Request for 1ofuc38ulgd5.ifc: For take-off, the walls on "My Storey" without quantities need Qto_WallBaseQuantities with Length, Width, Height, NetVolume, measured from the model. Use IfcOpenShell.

First a look at what the model holds.

```python
import ifcopenshell
import ifcopenshell.util.element
import ifcopenshell.util.unit

model = ifcopenshell.open("1ofuc38ulgd5.ifc")
print(model.schema)
for unit_type in ("LENGTHUNIT", "AREAUNIT", "VOLUMEUNIT"):
    print(unit_type, ifcopenshell.util.unit.calculate_unit_scale(model, unit_type))
storey = next(s for s in model.by_type("IfcBuildingStorey") if s.Name == "My Storey")
walls = [e for e in ifcopenshell.util.element.get_decomposition(storey) if e.is_a("IfcWall")]
for e in sorted(walls, key=lambda e: e.id()):
    print(e.id(), e.is_a(), e.Name, list(ifcopenshell.util.element.get_psets(e, qtos_only=True)), sep=" | ")
```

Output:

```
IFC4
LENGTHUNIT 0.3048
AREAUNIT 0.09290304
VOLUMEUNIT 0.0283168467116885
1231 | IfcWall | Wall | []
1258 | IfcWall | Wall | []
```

```python
import ifcopenshell
import ifcopenshell.api.pset
import ifcopenshell.geom
import ifcopenshell.util.element
import ifcopenshell.util.shape
import ifcopenshell.util.unit

model = ifcopenshell.open("1ofuc38ulgd5.ifc")
unit_scale = ifcopenshell.util.unit.calculate_unit_scale(model)
volume_scale = ifcopenshell.util.unit.calculate_unit_scale(model, "VOLUMEUNIT")
settings = ifcopenshell.geom.settings()

storey = next(s for s in model.by_type("IfcBuildingStorey") if s.Name == "My Storey")
walls = [e for e in ifcopenshell.util.element.get_decomposition(storey) if e.is_a("IfcWall")]

for e in sorted(walls, key=lambda e: e.id()):
    if ifcopenshell.util.element.get_psets(e, qtos_only=True, should_inherit=False):
        continue
    # Geometry comes back in metres, in the element's own axes.
    shape = ifcopenshell.geom.create_shape(settings, e)
    values = {
        "Length": ifcopenshell.util.shape.get_x(shape.geometry) / unit_scale,
        "Width": ifcopenshell.util.shape.get_y(shape.geometry) / unit_scale,
        "Height": ifcopenshell.util.shape.get_z(shape.geometry) / unit_scale,
        "NetVolume": ifcopenshell.util.shape.get_volume(shape.geometry) / volume_scale,
    }
    qto = ifcopenshell.api.pset.add_qto(model, product=e, name="Qto_WallBaseQuantities")
    ifcopenshell.api.pset.edit_qto(model, qto=qto, properties=values)
    print(e.id(), {k: round(v, 3) for k, v in values.items()})

model.write("1ofuc38ulgd5-out.ifc")
```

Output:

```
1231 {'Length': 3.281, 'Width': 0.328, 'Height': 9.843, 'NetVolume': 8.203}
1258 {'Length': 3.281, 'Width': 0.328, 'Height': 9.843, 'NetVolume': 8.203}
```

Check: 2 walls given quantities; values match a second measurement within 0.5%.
